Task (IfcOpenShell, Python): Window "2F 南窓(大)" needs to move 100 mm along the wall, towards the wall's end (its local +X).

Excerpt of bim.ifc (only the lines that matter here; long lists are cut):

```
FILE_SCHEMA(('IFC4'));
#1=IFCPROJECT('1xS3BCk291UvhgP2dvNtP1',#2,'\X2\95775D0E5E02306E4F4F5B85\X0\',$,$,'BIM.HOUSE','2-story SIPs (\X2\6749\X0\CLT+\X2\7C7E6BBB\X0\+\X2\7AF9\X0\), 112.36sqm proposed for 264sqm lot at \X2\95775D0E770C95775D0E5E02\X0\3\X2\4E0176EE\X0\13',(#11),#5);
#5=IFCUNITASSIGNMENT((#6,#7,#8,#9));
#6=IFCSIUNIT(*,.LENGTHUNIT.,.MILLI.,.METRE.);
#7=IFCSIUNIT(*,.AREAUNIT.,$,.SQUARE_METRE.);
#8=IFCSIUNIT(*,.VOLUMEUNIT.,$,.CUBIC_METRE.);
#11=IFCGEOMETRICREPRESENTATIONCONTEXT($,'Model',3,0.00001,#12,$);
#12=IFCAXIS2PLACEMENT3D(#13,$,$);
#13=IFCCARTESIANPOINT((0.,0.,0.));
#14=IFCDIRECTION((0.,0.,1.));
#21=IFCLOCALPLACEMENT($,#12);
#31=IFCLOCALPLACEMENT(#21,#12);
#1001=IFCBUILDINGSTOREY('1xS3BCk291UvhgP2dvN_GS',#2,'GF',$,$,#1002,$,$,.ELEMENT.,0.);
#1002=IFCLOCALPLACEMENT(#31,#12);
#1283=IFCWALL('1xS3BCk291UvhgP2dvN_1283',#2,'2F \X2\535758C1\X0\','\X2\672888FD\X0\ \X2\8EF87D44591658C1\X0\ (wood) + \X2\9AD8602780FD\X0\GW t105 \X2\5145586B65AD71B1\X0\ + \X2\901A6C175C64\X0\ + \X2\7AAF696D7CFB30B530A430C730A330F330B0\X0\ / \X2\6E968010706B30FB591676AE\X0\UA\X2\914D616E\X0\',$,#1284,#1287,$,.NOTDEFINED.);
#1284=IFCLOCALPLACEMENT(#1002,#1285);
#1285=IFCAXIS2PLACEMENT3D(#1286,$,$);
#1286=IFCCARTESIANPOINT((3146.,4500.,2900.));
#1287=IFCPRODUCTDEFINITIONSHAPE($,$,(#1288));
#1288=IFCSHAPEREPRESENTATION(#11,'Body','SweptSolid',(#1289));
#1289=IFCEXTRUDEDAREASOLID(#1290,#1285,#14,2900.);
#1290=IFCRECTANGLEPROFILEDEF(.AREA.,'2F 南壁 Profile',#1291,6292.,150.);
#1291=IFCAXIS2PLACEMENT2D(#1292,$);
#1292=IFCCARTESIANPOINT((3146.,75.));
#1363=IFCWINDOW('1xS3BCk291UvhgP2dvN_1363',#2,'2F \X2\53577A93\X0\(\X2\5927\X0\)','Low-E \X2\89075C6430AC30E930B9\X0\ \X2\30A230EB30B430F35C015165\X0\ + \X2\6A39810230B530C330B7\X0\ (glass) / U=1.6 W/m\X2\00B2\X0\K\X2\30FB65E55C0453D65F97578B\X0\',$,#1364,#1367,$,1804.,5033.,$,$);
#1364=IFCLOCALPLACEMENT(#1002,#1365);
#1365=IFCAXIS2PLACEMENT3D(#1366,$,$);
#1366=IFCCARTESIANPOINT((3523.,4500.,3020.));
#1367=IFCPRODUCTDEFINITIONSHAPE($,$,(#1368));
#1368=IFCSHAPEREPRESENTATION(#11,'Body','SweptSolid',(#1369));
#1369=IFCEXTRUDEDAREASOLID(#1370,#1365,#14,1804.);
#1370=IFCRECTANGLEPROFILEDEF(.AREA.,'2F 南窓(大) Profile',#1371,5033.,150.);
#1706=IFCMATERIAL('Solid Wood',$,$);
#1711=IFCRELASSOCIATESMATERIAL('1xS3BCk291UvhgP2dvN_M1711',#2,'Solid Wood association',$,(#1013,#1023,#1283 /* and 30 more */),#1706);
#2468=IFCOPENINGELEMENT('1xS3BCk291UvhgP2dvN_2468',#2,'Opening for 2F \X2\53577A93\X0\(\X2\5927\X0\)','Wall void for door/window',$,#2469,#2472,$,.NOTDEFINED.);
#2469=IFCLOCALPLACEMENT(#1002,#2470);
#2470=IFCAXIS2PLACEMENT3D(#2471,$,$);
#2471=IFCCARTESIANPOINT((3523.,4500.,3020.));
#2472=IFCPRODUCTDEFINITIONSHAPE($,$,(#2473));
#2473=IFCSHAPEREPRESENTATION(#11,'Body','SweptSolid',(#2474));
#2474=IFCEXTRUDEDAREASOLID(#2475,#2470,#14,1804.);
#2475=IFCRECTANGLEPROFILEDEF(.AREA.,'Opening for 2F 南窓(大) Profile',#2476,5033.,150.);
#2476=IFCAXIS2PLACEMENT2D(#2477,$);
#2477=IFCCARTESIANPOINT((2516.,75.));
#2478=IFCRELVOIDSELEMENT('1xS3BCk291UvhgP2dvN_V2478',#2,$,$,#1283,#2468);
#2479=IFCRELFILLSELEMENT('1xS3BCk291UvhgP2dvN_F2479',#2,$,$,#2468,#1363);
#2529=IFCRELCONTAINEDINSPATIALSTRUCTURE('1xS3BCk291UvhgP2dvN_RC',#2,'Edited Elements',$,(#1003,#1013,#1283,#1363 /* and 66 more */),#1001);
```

```python
import ifcopenshell
import ifcopenshell.api.geometry
import ifcopenshell.util.placement
import ifcopenshell.util.unit

model = ifcopenshell.open("bim.ifc")
unit_scale = ifcopenshell.util.unit.calculate_unit_scale(model)

window = model.by_guid("1xS3BCk291UvhgP2dvN_1363")
opening = window.FillsVoids[0].RelatingOpeningElement
wall = opening.VoidsElements[0].RelatingBuildingElement

wall_matrix = ifcopenshell.util.placement.get_local_placement(wall.ObjectPlacement)
shift = wall_matrix[:3, 0] * 0.1 / unit_scale
before = ifcopenshell.util.placement.get_local_placement(window.ObjectPlacement)[:3, 3].copy()

# The window is not placed relative to its opening, so move both.
for product in (opening, window):
    matrix = ifcopenshell.util.placement.get_local_placement(product.ObjectPlacement)
    matrix[:3, 3] += shift
    ifcopenshell.api.geometry.edit_object_placement(model, product=product, matrix=matrix, is_si=False)

after = ifcopenshell.util.placement.get_local_placement(window.ObjectPlacement)[:3, 3]
print("window moved by", (after - before).round(3) + 0.0)

model.write("bim_updated.ifc")
```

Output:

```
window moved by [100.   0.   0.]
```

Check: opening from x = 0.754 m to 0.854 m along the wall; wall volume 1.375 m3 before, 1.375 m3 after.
